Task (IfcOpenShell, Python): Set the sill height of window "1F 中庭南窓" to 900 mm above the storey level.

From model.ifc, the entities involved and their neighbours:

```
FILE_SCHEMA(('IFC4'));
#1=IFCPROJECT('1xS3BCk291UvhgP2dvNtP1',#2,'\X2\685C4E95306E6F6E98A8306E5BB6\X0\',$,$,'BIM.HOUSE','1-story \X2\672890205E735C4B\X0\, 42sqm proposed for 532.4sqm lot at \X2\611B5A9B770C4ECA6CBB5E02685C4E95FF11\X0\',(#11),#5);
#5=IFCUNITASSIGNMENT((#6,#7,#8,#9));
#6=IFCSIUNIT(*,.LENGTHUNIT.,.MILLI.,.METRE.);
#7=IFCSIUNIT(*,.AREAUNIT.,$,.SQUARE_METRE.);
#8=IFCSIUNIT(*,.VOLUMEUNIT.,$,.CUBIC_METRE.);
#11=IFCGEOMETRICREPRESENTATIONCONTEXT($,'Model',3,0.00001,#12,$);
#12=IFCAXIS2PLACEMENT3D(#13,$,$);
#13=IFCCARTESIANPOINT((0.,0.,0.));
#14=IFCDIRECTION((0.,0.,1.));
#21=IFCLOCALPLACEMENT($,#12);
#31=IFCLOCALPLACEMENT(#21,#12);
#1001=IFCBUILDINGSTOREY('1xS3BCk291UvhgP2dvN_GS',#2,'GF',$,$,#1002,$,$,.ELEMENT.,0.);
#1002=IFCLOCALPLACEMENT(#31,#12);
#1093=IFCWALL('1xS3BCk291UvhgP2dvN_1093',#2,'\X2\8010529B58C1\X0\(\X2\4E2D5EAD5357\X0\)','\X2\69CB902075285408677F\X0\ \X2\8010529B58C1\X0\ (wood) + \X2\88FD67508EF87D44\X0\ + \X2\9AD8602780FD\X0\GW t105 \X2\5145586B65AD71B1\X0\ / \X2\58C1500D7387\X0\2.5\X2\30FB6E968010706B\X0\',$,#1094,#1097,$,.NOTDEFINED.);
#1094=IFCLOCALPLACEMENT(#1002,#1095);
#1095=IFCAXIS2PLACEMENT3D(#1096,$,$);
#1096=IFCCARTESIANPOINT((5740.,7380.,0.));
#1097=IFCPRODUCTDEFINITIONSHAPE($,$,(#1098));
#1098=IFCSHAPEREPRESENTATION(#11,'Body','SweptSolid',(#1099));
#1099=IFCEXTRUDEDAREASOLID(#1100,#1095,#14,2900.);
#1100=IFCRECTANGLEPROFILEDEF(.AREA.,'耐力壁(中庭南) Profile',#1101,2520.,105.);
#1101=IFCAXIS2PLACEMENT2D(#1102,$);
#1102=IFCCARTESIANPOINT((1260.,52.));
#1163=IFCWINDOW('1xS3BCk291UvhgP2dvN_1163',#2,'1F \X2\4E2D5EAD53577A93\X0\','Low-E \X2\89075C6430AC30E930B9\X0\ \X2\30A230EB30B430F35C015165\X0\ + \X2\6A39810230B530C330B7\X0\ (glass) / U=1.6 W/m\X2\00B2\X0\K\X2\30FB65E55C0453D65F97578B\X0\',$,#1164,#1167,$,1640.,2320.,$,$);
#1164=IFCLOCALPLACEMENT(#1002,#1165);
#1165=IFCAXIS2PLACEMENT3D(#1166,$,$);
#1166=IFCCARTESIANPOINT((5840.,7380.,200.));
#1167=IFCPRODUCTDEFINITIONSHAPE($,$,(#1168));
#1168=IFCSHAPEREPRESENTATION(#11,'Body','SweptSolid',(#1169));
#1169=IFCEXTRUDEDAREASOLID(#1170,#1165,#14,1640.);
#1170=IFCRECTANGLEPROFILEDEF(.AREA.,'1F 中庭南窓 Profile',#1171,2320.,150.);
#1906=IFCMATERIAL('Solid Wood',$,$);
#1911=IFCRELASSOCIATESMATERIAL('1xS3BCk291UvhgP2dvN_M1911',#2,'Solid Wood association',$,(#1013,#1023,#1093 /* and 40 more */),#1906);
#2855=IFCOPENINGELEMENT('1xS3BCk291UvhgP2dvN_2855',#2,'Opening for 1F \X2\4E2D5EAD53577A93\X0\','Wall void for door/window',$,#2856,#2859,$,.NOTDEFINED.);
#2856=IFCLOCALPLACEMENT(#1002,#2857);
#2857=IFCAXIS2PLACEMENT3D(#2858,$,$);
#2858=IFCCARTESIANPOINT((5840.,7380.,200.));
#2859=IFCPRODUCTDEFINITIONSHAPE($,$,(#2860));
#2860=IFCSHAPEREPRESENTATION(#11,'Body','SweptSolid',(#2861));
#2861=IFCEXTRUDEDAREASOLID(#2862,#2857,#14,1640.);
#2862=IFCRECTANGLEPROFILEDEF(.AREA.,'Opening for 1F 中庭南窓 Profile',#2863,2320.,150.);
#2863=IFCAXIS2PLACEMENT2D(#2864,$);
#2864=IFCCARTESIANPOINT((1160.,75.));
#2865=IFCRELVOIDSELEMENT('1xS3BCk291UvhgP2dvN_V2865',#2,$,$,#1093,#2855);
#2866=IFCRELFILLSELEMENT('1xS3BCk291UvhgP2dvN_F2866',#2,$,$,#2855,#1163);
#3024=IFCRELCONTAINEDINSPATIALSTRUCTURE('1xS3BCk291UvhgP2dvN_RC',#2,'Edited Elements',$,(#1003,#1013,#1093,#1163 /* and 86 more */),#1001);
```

```python
import numpy as np
import ifcopenshell
import ifcopenshell.api.geometry
import ifcopenshell.geom
import ifcopenshell.util.element
import ifcopenshell.util.placement
import ifcopenshell.util.shape
import ifcopenshell.util.unit

model = ifcopenshell.open("model.ifc")
unit_scale = ifcopenshell.util.unit.calculate_unit_scale(model)

window = model.by_guid("1xS3BCk291UvhgP2dvN_1163")
opening = window.FillsVoids[0].RelatingOpeningElement
storey = ifcopenshell.util.element.get_container(window, ifc_class="IfcBuildingStorey")
level = ifcopenshell.util.placement.get_local_placement(storey.ObjectPlacement)[2, 3]

# The opening's origin need not be at the sill, so measure its lowest point.
shape = ifcopenshell.geom.create_shape(ifcopenshell.geom.settings(), opening)
bottom = ifcopenshell.util.shape.get_shape_bottom_elevation(shape, shape.geometry) / unit_scale
dz = level + 0.9 / unit_scale - bottom

shift = np.array([0.0, 0.0, dz])
# The window is not placed relative to its opening, so move both.
for product in (opening, window):
    matrix = ifcopenshell.util.placement.get_local_placement(product.ObjectPlacement)
    matrix[:3, 3] += shift
    ifcopenshell.api.geometry.edit_object_placement(model, product=product, matrix=matrix, is_si=False)

print(f"moved by {dz * unit_scale:+.3f} m")

model.write("model_v2.ifc")
```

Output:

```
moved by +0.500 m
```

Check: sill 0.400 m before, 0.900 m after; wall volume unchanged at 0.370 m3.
